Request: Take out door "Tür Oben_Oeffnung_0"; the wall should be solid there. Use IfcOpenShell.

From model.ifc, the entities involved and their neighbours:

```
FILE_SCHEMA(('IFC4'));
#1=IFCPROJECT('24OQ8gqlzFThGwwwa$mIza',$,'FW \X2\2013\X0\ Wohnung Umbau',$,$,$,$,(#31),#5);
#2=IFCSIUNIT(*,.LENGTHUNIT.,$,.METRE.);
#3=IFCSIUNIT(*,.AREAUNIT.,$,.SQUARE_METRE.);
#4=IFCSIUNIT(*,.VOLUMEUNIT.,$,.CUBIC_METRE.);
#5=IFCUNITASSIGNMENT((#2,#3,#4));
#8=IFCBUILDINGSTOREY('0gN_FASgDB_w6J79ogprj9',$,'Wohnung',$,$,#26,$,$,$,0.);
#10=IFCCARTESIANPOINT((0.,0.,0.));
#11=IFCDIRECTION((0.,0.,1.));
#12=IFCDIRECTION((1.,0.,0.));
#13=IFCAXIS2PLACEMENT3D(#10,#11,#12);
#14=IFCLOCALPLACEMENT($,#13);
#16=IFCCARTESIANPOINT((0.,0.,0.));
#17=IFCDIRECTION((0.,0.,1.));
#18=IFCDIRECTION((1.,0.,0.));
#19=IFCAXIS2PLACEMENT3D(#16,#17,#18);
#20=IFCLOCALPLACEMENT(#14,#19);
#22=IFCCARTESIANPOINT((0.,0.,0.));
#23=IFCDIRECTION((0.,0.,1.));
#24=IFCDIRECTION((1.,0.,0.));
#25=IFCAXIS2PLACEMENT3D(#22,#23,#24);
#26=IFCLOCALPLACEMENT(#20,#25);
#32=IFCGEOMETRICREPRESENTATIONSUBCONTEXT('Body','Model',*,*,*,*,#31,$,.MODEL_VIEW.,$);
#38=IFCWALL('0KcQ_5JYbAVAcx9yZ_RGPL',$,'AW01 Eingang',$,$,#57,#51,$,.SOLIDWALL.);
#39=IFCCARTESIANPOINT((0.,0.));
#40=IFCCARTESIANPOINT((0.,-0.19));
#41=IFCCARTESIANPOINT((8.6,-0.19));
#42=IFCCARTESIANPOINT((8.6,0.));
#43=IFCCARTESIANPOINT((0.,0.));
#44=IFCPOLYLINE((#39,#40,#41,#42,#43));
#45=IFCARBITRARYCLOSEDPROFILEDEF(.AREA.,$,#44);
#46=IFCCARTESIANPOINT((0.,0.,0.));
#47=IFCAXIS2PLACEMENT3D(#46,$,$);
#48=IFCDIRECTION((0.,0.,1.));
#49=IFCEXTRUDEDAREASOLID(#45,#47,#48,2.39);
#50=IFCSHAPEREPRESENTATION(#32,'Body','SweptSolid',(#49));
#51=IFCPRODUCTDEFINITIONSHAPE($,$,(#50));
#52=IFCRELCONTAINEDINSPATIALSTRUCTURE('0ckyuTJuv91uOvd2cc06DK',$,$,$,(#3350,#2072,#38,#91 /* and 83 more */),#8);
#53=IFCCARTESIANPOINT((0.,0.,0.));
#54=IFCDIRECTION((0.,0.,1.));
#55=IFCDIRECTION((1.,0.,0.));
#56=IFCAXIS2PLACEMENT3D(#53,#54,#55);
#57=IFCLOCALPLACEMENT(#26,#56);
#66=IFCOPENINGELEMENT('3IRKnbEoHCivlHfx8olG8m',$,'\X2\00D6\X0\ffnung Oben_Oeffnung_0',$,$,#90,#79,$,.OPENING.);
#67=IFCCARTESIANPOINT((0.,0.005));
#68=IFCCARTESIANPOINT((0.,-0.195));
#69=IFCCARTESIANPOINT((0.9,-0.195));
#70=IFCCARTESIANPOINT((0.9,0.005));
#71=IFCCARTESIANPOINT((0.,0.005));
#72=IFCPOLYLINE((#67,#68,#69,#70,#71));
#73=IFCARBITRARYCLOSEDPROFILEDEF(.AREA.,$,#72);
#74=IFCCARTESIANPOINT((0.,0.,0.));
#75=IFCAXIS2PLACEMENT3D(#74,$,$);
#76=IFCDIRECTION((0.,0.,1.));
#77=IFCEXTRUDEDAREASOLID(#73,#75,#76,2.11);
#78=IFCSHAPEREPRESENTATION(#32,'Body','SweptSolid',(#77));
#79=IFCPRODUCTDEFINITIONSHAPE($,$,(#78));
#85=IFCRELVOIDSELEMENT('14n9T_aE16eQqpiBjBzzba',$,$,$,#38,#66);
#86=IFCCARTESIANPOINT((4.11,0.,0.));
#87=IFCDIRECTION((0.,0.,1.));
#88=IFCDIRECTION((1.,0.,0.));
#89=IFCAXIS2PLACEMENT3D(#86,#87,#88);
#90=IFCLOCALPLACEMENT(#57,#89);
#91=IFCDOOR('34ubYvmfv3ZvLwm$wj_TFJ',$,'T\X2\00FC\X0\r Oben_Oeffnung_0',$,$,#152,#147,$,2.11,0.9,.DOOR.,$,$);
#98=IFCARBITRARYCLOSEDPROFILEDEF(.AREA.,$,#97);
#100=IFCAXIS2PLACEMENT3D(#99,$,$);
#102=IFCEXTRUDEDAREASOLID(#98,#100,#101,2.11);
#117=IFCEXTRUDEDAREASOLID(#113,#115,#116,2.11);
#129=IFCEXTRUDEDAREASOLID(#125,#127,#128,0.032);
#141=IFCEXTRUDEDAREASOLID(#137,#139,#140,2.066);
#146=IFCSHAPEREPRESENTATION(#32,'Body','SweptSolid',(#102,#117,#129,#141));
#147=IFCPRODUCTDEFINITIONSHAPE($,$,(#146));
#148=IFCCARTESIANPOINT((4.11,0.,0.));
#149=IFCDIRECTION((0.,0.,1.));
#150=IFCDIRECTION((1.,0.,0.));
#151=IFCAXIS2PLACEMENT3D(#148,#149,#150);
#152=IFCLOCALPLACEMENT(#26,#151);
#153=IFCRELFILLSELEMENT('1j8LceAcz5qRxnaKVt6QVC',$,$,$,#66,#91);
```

```python
import ifcopenshell
import ifcopenshell.api.feature
import ifcopenshell.api.root
import ifcopenshell.geom
import ifcopenshell.util.shape

model = ifcopenshell.open("model.ifc")
settings = ifcopenshell.geom.settings()


def volume(element):
    """Net volume in cubic metres, openings subtracted."""
    shape = ifcopenshell.geom.create_shape(settings, element)
    return ifcopenshell.util.shape.get_volume(shape.geometry)


door = model.by_guid("34ubYvmfv3ZvLwm$wj_TFJ")
opening = door.FillsVoids[0].RelatingOpeningElement
wall = opening.VoidsElements[0].RelatingBuildingElement
before = volume(wall)

ifcopenshell.api.root.remove_product(model, product=door)
ifcopenshell.api.feature.remove_feature(model, feature=opening)

after = volume(wall)

print(f"wall volume {before:.3f} -> {after:.3f} m3")

model.write("model_updated.ifc")
```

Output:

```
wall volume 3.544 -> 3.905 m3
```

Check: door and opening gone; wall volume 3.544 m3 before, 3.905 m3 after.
